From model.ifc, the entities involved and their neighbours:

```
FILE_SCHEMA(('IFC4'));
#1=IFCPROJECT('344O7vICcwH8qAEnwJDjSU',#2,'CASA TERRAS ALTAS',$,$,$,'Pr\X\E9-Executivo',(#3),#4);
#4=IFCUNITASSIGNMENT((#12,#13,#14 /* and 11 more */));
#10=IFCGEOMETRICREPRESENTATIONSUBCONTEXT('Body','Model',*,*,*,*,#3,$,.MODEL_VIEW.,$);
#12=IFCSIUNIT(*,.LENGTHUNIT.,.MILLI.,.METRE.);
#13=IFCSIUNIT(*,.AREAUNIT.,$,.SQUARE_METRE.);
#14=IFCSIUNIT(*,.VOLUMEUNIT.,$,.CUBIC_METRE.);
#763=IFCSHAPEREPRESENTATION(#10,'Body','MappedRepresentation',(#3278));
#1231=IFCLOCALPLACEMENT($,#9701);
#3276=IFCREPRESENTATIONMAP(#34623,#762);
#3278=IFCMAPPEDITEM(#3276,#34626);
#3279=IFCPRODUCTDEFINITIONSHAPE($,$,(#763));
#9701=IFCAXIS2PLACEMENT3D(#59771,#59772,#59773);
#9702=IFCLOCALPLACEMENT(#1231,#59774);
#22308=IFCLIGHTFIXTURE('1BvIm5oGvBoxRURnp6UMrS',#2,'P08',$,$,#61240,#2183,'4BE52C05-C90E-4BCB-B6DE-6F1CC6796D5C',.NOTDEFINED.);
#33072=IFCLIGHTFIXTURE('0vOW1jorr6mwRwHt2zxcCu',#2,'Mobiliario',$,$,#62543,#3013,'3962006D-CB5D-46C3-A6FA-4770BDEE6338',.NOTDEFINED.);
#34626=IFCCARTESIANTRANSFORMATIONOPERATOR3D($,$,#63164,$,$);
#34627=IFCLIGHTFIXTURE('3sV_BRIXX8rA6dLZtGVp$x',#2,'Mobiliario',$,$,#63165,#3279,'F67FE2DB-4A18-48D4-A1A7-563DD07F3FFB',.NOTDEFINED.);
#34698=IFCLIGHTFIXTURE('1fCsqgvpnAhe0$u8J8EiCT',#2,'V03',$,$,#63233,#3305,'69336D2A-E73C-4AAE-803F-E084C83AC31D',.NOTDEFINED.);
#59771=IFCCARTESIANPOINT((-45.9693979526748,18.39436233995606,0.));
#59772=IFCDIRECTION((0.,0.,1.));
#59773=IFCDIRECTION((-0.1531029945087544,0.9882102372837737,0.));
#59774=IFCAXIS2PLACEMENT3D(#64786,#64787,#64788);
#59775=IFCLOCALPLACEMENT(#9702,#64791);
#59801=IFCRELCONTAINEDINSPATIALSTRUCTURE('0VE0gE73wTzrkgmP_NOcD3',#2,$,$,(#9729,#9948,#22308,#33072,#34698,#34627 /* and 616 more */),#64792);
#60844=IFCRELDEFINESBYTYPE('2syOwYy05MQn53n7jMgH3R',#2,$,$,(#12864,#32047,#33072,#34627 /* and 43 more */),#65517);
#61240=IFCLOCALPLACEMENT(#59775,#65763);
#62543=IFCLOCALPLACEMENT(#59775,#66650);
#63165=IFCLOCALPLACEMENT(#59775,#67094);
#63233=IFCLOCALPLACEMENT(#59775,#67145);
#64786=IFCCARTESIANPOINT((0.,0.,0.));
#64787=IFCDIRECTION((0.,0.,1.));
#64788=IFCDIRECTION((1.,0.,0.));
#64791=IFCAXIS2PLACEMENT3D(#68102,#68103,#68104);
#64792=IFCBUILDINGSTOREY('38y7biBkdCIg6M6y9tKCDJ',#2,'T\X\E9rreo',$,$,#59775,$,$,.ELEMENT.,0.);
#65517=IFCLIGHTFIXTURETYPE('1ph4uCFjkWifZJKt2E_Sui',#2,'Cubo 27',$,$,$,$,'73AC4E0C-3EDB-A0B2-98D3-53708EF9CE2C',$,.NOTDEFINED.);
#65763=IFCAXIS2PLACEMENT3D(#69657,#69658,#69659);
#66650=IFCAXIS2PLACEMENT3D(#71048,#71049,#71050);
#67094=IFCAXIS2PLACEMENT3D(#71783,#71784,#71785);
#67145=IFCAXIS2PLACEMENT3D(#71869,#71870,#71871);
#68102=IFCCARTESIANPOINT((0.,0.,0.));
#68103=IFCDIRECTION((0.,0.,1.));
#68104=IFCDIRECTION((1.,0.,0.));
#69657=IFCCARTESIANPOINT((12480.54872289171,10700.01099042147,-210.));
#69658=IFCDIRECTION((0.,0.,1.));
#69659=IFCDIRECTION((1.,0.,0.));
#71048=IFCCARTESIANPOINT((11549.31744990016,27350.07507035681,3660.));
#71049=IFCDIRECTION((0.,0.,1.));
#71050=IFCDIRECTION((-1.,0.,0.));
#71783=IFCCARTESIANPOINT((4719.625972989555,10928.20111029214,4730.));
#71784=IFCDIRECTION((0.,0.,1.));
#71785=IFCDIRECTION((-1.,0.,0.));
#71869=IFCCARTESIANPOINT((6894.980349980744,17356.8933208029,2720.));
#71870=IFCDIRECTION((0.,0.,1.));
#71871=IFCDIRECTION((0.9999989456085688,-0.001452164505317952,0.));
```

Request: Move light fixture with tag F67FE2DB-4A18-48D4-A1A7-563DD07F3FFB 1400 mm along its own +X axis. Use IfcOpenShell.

```python
import ifcopenshell
import ifcopenshell.api.geometry
import ifcopenshell.util.placement
import ifcopenshell.util.unit

model = ifcopenshell.open("model.ifc")
unit_scale = ifcopenshell.util.unit.calculate_unit_scale(model)

item = model.by_id(34627)
matrix = ifcopenshell.util.placement.get_local_placement(item.ObjectPlacement)
matrix[:3, 3] += matrix[:3, 0] * 1.4 / unit_scale
ifcopenshell.api.geometry.edit_object_placement(model, product=item, matrix=matrix, is_si=False)

print(ifcopenshell.util.placement.get_local_placement(item.ObjectPlacement).round(3) + 0.0)

model.write("model-out.ifc")
```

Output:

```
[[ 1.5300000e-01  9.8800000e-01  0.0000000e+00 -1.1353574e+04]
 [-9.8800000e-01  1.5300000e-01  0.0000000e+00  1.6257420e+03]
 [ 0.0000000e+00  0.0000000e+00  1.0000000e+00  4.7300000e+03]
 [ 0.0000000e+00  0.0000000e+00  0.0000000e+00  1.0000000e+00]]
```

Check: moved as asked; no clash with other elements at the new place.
